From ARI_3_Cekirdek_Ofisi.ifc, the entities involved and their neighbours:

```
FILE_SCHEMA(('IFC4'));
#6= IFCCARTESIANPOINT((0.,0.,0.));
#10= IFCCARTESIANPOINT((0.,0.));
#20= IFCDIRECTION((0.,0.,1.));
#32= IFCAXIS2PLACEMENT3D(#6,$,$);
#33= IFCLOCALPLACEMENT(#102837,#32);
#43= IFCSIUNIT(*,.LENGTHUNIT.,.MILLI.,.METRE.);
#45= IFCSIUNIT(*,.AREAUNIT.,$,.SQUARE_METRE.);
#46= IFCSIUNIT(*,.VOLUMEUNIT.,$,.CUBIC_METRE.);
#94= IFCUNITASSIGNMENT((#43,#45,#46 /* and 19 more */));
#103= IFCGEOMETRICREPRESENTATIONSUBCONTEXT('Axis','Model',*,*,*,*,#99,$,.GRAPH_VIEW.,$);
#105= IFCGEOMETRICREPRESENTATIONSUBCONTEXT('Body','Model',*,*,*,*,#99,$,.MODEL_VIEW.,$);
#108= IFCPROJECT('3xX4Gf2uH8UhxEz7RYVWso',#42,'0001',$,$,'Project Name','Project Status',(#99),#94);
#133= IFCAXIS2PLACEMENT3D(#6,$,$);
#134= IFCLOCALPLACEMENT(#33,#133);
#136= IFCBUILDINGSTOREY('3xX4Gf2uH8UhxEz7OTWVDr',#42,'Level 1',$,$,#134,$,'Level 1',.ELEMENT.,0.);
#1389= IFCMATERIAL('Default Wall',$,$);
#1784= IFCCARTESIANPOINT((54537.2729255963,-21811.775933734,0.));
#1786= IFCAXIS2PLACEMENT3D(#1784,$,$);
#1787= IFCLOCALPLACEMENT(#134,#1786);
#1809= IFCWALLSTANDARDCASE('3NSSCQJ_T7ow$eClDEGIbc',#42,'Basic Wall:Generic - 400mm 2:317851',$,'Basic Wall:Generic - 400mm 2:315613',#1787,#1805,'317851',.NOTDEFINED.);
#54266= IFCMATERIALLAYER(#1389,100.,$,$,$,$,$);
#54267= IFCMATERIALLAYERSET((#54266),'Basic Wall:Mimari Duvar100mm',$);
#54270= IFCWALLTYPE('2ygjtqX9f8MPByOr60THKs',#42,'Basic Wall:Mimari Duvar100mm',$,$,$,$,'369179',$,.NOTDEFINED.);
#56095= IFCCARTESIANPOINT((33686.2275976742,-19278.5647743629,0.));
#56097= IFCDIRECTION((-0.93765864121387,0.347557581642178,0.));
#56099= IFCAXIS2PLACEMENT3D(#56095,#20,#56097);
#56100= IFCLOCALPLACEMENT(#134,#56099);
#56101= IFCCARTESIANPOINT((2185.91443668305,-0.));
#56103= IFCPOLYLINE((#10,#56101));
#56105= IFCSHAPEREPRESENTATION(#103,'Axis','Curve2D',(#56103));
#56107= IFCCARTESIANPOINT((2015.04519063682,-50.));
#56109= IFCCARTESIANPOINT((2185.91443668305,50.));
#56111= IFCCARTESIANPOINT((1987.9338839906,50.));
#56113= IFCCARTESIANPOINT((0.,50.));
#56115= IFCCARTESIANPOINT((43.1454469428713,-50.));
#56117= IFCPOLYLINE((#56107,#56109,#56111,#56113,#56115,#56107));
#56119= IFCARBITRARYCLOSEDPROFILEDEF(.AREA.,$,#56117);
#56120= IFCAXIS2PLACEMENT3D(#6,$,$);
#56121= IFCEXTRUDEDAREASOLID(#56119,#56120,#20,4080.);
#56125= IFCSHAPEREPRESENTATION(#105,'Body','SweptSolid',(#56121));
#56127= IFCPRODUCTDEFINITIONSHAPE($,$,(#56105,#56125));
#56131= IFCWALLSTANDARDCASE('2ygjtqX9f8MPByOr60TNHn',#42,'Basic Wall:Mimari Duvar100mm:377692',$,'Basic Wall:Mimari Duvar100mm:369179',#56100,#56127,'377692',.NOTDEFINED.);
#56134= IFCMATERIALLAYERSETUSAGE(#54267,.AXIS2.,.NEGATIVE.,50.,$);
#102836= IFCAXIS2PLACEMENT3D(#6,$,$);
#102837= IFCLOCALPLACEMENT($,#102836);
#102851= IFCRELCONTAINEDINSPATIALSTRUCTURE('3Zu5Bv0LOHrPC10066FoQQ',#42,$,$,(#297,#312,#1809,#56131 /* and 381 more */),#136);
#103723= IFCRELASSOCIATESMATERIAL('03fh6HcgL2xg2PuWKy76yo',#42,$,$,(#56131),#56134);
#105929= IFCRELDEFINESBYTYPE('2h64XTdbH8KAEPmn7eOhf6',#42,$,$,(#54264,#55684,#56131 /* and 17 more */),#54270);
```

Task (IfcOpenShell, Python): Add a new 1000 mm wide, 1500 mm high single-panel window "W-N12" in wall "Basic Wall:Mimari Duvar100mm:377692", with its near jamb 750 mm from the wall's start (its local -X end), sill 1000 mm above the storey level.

```python
import numpy as np
import ifcopenshell
import ifcopenshell.api.feature
import ifcopenshell.api.geometry
import ifcopenshell.api.root
import ifcopenshell.api.spatial
import ifcopenshell.geom
import ifcopenshell.util.element
import ifcopenshell.util.placement
import ifcopenshell.util.representation
import ifcopenshell.util.shape
import ifcopenshell.util.unit

model = ifcopenshell.open("ARI_3_Cekirdek_Ofisi.ifc")
unit_scale = ifcopenshell.util.unit.calculate_unit_scale(model)
settings = ifcopenshell.geom.settings()


def volume(element):
    """Net volume in cubic metres, openings subtracted."""
    shape = ifcopenshell.geom.create_shape(settings, element)
    return ifcopenshell.util.shape.get_volume(shape.geometry)


wall = model.by_guid("2ygjtqX9f8MPByOr60TNHn")
storey = ifcopenshell.util.element.get_container(wall, ifc_class="IfcBuildingStorey")
context = ifcopenshell.util.representation.get_context(model, "Model", "Body", "MODEL_VIEW")
before = volume(wall)

width, height, from_end, sill = 1, 1.5, 0.75, 1  # metres

# The wall runs along its own X axis, and the end named is its -X end.
wall_shape = ifcopenshell.geom.create_shape(settings, wall)
x, y, z = ifcopenshell.util.shape.get_vertices(wall_shape.geometry).T
start = x.min() + from_end
face, thickness = float(y.min()), float(y.max() - y.min())
wall_matrix = ifcopenshell.util.placement.get_local_placement(wall.ObjectPlacement)
level = ifcopenshell.util.placement.get_local_placement(storey.ObjectPlacement)[2, 3]


def in_wall(x, y):
    """Placement at x, y metres in the wall's axes, at sill height."""
    matrix = wall_matrix.copy()
    matrix[:, 3] = wall_matrix @ np.array([x / unit_scale, y / unit_scale, 0.0, 1.0])
    matrix[2, 3] = level + sill / unit_scale
    return matrix


# Opening: a box that overshoots both wall faces by 50 mm.
opening = ifcopenshell.api.root.create_entity(model, ifc_class="IfcOpeningElement", predefined_type="OPENING")
box = ifcopenshell.api.geometry.add_wall_representation(
    model, context=context, length=width, height=height, thickness=thickness + 0.1
)
ifcopenshell.api.geometry.assign_representation(model, product=opening, representation=box)
ifcopenshell.api.geometry.edit_object_placement(model, product=opening, matrix=in_wall(start, face - 0.05), is_si=False)
ifcopenshell.api.feature.add_feature(model, feature=opening, element=wall)

window = ifcopenshell.api.root.create_entity(model, ifc_class="IfcWindow", name="W-N12", predefined_type="WINDOW")
window.OverallWidth, window.OverallHeight = width / unit_scale, height / unit_scale
window.PartitioningType = "SINGLE_PANEL"
body = ifcopenshell.api.geometry.add_window_representation(
    model,
    context=context,
    overall_width=window.OverallWidth,
    overall_height=window.OverallHeight,
    partition_type="SINGLE_PANEL",
)
ifcopenshell.api.geometry.assign_representation(model, product=window, representation=body)
ifcopenshell.api.spatial.assign_container(model, products=[window], relating_structure=storey)
ifcopenshell.api.feature.add_filling(model, opening=opening, element=window)

# Centre the window in the wall's thickness.
ifcopenshell.api.geometry.edit_object_placement(model, product=window, matrix=in_wall(start, face), is_si=False)
window_shape = ifcopenshell.geom.create_shape(settings, window)
depth = ifcopenshell.util.shape.get_vertices(window_shape.geometry)[:, 1]
offset = face + thickness / 2 - (depth.min() + depth.max()) / 2
ifcopenshell.api.geometry.edit_object_placement(model, product=window, matrix=in_wall(start, offset), is_si=False)

after = volume(wall)

print(f"wall volume {before:.3f} -> {after:.3f} m3")

model.write("ARI_3_Cekirdek_Ofisi_v2.ifc")
```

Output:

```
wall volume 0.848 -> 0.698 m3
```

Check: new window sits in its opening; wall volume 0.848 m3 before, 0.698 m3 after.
